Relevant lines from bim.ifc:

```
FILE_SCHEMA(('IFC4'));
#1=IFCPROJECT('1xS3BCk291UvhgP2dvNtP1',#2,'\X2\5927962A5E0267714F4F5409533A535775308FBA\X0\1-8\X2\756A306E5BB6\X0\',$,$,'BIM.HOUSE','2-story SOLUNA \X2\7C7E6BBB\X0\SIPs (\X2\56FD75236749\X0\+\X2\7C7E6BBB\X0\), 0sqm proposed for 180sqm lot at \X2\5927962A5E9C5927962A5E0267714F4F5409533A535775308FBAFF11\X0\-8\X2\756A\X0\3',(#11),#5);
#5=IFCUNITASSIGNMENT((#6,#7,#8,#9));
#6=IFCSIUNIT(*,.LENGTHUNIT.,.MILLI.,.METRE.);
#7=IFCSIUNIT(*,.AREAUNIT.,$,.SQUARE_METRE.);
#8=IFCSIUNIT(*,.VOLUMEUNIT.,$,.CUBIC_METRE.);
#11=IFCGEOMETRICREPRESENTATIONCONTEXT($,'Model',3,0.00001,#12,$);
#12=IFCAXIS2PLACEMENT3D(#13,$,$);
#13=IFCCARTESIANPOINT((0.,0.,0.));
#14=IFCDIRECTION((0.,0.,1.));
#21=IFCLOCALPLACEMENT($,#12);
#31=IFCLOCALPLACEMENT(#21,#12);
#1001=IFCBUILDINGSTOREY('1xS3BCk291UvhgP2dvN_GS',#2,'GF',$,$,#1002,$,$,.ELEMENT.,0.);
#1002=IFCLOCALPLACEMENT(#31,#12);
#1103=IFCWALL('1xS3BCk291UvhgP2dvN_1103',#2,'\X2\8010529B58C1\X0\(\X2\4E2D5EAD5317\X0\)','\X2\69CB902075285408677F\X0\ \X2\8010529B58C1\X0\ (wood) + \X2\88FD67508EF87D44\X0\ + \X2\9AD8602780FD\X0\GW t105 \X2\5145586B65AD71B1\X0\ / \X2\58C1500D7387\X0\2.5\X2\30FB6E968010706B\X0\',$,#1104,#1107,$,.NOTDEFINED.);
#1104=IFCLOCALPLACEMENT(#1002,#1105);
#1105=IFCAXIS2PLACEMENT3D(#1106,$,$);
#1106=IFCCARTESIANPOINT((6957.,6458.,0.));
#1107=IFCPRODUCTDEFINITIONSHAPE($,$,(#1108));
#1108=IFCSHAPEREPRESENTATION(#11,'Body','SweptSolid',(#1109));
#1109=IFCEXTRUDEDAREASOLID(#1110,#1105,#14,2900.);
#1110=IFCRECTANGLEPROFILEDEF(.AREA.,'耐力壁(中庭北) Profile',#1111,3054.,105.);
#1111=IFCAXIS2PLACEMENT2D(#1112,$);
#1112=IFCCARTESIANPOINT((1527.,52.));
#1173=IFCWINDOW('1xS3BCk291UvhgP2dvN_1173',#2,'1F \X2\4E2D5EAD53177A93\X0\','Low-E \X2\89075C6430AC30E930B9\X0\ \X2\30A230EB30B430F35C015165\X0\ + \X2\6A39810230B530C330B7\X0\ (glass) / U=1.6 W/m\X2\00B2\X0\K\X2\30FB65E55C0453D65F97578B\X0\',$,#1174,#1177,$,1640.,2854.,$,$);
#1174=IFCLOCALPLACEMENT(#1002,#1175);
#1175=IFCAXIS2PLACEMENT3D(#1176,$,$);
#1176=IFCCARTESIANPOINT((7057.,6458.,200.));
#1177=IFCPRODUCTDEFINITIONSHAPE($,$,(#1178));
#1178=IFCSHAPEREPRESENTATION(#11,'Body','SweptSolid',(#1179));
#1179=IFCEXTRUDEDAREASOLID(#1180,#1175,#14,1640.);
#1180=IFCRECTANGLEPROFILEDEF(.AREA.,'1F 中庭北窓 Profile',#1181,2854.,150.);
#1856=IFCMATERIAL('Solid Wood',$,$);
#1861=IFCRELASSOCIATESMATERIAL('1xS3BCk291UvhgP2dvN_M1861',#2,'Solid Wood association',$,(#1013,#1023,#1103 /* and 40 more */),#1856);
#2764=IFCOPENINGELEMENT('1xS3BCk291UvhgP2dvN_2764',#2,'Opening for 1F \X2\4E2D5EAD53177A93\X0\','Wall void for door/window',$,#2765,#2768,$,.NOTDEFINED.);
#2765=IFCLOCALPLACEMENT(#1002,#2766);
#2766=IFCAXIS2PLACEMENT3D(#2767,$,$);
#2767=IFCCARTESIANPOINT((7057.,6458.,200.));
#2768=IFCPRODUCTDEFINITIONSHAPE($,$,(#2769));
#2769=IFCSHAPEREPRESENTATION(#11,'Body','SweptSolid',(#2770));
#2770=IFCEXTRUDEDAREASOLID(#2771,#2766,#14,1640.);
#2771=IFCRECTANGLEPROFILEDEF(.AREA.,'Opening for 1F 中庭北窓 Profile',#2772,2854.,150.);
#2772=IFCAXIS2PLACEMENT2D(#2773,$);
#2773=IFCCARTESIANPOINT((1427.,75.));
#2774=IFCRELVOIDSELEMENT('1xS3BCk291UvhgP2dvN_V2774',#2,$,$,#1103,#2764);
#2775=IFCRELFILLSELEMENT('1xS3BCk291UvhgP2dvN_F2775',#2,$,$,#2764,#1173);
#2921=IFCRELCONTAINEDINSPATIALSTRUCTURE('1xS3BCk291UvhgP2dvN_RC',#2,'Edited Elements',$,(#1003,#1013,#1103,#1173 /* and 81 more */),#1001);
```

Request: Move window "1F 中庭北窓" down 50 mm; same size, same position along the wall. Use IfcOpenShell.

```python
import numpy as np
import ifcopenshell
import ifcopenshell.api.geometry
import ifcopenshell.util.placement
import ifcopenshell.util.unit

model = ifcopenshell.open("bim.ifc")
unit_scale = ifcopenshell.util.unit.calculate_unit_scale(model)

window = model.by_guid("1xS3BCk291UvhgP2dvN_1173")
opening = window.FillsVoids[0].RelatingOpeningElement
dz = -0.05 / unit_scale

shift = np.array([0.0, 0.0, dz])
# The window is not placed relative to its opening, so move both.
for product in (opening, window):
    matrix = ifcopenshell.util.placement.get_local_placement(product.ObjectPlacement)
    matrix[:3, 3] += shift
    ifcopenshell.api.geometry.edit_object_placement(model, product=product, matrix=matrix, is_si=False)

print(f"moved by {dz * unit_scale:+.3f} m")

model.write("bim-out.ifc")
```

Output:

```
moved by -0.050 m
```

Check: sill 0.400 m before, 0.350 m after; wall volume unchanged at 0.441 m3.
